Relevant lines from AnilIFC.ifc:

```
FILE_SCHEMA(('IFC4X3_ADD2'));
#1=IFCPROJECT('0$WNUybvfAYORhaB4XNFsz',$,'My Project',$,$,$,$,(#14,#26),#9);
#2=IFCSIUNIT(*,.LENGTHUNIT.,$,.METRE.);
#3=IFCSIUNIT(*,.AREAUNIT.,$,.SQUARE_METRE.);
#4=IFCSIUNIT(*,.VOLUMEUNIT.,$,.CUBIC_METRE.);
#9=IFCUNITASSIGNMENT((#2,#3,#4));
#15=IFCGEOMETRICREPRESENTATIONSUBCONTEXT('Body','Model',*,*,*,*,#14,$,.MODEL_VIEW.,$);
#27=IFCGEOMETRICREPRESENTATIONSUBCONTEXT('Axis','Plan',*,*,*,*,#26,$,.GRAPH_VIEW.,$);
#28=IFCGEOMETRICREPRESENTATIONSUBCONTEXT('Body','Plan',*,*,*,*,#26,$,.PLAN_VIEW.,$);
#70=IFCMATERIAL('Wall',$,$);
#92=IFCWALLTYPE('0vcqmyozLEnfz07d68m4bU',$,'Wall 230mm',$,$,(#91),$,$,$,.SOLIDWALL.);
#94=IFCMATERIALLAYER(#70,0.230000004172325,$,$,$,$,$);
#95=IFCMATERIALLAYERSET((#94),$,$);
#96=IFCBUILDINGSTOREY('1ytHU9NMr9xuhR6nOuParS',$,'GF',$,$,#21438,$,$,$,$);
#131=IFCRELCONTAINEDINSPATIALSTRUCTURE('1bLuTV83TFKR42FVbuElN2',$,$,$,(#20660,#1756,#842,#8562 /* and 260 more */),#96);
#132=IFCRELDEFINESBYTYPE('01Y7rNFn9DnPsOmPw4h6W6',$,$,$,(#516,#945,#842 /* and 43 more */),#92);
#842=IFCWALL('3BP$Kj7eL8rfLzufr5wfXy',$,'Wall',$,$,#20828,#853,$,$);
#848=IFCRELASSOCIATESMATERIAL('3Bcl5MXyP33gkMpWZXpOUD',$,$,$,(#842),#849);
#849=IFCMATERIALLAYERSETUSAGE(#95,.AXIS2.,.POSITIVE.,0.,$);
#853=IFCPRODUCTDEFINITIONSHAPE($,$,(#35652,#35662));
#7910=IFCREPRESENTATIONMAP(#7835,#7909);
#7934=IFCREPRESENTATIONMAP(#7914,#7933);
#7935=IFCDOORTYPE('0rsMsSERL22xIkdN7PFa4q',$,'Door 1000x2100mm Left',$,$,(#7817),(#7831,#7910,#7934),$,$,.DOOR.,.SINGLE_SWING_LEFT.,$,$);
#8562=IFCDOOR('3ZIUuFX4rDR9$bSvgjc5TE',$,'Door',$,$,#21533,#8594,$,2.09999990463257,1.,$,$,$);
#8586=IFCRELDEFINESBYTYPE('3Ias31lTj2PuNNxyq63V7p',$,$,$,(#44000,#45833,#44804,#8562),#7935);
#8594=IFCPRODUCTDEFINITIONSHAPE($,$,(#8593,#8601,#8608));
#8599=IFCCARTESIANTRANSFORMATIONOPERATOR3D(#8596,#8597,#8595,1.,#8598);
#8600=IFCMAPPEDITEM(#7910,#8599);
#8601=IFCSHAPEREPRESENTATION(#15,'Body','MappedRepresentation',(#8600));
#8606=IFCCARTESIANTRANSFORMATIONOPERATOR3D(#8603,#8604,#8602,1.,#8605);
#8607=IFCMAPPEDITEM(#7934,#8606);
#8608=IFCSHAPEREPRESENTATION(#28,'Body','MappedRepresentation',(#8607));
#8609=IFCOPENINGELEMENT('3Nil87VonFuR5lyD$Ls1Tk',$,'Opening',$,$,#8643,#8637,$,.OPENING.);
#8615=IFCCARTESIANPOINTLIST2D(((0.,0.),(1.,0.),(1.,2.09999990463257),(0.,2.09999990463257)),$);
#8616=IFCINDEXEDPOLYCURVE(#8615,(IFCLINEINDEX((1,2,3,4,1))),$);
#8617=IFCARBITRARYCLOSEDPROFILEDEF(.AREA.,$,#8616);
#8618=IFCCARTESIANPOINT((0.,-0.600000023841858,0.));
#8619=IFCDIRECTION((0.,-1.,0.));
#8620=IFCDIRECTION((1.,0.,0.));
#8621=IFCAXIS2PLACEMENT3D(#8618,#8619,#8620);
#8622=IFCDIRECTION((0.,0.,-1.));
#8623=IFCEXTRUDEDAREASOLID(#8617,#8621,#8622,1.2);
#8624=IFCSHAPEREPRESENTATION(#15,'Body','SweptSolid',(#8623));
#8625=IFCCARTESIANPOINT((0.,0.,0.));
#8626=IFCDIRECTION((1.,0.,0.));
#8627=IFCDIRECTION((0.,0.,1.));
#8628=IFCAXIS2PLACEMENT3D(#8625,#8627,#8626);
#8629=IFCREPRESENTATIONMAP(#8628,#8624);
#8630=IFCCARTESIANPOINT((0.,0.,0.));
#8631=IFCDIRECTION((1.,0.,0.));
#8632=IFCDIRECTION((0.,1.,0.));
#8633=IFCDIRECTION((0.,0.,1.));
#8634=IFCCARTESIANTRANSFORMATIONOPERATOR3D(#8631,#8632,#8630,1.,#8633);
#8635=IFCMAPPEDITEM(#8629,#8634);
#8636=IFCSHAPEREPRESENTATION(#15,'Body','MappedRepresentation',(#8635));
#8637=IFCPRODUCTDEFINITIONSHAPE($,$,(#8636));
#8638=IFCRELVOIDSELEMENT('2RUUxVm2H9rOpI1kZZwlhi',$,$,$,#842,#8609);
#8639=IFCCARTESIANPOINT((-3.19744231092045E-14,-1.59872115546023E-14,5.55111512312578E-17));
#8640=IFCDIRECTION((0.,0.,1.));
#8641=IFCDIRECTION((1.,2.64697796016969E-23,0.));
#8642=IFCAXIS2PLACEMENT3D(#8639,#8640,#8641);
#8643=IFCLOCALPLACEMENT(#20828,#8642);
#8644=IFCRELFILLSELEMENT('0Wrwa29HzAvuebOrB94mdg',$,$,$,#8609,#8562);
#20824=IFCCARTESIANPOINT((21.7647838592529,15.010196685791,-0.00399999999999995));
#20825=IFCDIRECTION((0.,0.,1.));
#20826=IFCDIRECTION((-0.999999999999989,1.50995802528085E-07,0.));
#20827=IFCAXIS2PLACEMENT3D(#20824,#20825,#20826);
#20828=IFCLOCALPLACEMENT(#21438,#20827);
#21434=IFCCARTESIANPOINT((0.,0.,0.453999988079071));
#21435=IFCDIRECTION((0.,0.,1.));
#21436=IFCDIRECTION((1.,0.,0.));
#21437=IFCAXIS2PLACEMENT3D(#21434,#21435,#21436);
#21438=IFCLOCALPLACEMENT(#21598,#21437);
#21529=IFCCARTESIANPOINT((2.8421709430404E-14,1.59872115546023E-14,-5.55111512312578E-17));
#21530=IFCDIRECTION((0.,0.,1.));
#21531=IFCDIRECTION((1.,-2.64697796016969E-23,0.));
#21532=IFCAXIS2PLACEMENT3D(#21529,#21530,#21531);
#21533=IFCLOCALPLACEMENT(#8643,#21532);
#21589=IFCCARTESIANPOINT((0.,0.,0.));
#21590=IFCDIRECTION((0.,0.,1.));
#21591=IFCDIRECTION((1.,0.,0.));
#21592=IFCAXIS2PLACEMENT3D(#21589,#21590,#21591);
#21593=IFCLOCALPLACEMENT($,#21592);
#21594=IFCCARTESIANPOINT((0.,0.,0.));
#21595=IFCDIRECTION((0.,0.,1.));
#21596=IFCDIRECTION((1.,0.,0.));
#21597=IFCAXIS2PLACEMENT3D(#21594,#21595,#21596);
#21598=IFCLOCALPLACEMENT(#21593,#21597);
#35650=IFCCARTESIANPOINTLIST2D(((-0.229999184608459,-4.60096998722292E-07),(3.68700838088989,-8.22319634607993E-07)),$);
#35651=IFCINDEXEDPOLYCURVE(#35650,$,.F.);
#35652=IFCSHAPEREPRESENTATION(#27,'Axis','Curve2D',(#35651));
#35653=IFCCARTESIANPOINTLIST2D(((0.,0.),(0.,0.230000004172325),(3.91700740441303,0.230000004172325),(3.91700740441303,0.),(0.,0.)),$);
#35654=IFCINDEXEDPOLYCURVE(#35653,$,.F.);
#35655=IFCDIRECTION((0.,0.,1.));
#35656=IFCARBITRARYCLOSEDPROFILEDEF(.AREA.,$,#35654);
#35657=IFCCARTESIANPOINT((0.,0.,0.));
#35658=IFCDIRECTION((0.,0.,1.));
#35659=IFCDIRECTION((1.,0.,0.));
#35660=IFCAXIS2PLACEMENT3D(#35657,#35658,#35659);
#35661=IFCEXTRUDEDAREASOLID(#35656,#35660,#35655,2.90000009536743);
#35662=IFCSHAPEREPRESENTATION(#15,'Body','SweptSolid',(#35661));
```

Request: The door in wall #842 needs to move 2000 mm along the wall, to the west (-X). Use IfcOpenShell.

```python
import ifcopenshell
import ifcopenshell.api.geometry
import ifcopenshell.util.placement
import ifcopenshell.util.unit

model = ifcopenshell.open("AnilIFC.ifc")
unit_scale = ifcopenshell.util.unit.calculate_unit_scale(model)

door = model.by_id(8562)
opening = door.FillsVoids[0].RelatingOpeningElement
wall = opening.VoidsElements[0].RelatingBuildingElement

wall_matrix = ifcopenshell.util.placement.get_local_placement(wall.ObjectPlacement)
shift = wall_matrix[:3, 0] * 2 / unit_scale
before = ifcopenshell.util.placement.get_local_placement(door.ObjectPlacement)[:3, 3].copy()

# The door is placed relative to its opening, so it follows when the opening moves.
matrix = ifcopenshell.util.placement.get_local_placement(opening.ObjectPlacement)
matrix[:3, 3] += shift
ifcopenshell.api.geometry.edit_object_placement(
    model, product=opening, matrix=matrix, is_si=False, should_transform_children=True
)

after = ifcopenshell.util.placement.get_local_placement(door.ObjectPlacement)[:3, 3]
print("door moved by", (after - before).round(3) + 0.0)

model.write("AnilIFC_edited.ifc")
```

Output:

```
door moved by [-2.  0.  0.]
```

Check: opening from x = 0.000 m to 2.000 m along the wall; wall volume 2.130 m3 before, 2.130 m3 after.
